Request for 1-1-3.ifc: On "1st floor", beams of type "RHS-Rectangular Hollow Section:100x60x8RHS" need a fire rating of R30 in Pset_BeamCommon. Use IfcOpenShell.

First a look at what the model holds.

```python
import ifcopenshell
import ifcopenshell.util.element

model = ifcopenshell.open("1-1-3.ifc")
print(model.schema)
storey = next(s for s in model.by_type("IfcBuildingStorey") if s.Name == "1st floor")
beams = [e for e in ifcopenshell.util.element.get_decomposition(storey) if e.is_a("IfcBeam")]
seen = {}
for e in beams:
    element_type = ifcopenshell.util.element.get_type(e)
    key = (element_type.Name if element_type != e and element_type else None, ifcopenshell.util.element.get_pset(e, "Pset_BeamCommon", "FireRating"))
    seen[key] = seen.get(key, 0) + 1
for (name, value), count in sorted(seen.items(), key=str):
    print(count, "x", name, "|", value)
```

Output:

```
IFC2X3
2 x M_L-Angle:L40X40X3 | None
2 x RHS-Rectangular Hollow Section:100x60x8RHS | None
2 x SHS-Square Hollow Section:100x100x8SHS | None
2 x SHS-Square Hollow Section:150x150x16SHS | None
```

```python
import ifcopenshell
import ifcopenshell.api.pset
import ifcopenshell.util.element

model = ifcopenshell.open("1-1-3.ifc")

storey = next(s for s in model.by_type("IfcBuildingStorey") if s.Name == "1st floor")
beams = [e for e in ifcopenshell.util.element.get_decomposition(storey) if e.is_a("IfcBeam")]

count = 0
for e in beams:
    element_type = ifcopenshell.util.element.get_type(e)
    if element_type in (None, e) or element_type.Name != "RHS-Rectangular Hollow Section:100x60x8RHS":
        continue
    # add_pset returns the element's existing set when there is one.
    pset = ifcopenshell.api.pset.add_pset(model, product=e, name="Pset_BeamCommon")
    ifcopenshell.api.pset.edit_pset(model, pset=pset, properties={"FireRating": "R30"})
    count += 1

print(count, "beams updated")

model.write("1-1-3_edited.ifc")
```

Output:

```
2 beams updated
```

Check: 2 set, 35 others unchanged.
